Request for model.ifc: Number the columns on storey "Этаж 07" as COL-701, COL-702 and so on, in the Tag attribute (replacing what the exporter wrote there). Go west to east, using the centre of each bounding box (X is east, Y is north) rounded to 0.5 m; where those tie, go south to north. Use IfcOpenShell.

First a look at what the model holds.

```python
import ifcopenshell
import ifcopenshell.util.element
import ifcopenshell.util.placement

model = ifcopenshell.open("model.ifc")
print(model.schema)
storey = next(s for s in model.by_type("IfcBuildingStorey") if s.Name == "Этаж 07")
columns = [e for e in ifcopenshell.util.element.get_decomposition(storey) if e.is_a("IfcColumn")]
for e in sorted(columns, key=lambda e: e.id()):
    origin = ifcopenshell.util.placement.get_local_placement(e.ObjectPlacement)[:3, 3]
    print(e.id(), e.Tag, e.Name, origin.round(2) + 0.0, sep=" | ")
```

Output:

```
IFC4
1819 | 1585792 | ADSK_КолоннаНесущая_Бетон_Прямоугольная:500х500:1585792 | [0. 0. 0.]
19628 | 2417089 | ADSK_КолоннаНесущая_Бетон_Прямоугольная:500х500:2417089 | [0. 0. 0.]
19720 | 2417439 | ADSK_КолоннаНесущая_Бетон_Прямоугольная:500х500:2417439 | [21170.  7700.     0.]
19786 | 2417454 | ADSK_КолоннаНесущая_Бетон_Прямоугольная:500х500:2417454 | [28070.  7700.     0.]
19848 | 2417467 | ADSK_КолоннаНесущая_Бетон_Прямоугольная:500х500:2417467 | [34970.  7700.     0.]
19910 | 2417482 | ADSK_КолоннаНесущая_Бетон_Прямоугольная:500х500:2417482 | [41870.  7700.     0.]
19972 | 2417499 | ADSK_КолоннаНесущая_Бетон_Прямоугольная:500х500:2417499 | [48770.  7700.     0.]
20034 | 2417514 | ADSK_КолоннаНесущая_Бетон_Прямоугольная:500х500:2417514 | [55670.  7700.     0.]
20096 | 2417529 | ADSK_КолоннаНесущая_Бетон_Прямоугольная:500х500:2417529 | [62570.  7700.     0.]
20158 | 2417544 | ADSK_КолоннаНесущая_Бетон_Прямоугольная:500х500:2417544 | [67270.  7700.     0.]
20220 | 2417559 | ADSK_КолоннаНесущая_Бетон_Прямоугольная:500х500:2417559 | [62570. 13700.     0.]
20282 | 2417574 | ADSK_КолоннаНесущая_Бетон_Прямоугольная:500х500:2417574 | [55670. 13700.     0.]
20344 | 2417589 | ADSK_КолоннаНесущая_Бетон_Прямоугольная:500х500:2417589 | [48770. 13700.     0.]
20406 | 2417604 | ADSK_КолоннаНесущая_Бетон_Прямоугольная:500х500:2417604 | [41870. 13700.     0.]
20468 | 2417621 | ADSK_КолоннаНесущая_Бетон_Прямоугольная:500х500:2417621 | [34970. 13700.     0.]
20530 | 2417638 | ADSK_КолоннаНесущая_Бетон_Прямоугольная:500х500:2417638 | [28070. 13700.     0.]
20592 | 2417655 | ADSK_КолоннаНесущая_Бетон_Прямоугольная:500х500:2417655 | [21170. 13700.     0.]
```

```python
import ifcopenshell
import ifcopenshell.geom
import ifcopenshell.util.element
import ifcopenshell.util.shape

model = ifcopenshell.open("model.ifc")
settings = ifcopenshell.geom.settings()
settings.set("use-world-coords", True)


def centre(element):
    shape = ifcopenshell.geom.create_shape(settings, element)
    return ifcopenshell.util.shape.get_bbox_centroid(shape.geometry)


storey = next(s for s in model.by_type("IfcBuildingStorey") if s.Name == "Этаж 07")
columns = [e for e in ifcopenshell.util.element.get_decomposition(storey) if e.is_a("IfcColumn")]

# Insertion points can sit at a corner or the storey origin, so sort by the geometry (in metres).
centres = {e: centre(e) for e in columns}
columns.sort(key=lambda e: (round(centres[e][0] / 0.5), centres[e][1]))

for i, e in enumerate(columns, start=1):
    number = f"COL-7{i:02d}"
    e.Tag = number
    print(e.id(), number)

model.write("model_updated.ifc")
```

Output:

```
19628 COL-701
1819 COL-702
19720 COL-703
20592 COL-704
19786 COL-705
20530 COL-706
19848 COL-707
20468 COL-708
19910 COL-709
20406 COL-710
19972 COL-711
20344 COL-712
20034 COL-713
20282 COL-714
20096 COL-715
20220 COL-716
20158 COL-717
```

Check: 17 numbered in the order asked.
